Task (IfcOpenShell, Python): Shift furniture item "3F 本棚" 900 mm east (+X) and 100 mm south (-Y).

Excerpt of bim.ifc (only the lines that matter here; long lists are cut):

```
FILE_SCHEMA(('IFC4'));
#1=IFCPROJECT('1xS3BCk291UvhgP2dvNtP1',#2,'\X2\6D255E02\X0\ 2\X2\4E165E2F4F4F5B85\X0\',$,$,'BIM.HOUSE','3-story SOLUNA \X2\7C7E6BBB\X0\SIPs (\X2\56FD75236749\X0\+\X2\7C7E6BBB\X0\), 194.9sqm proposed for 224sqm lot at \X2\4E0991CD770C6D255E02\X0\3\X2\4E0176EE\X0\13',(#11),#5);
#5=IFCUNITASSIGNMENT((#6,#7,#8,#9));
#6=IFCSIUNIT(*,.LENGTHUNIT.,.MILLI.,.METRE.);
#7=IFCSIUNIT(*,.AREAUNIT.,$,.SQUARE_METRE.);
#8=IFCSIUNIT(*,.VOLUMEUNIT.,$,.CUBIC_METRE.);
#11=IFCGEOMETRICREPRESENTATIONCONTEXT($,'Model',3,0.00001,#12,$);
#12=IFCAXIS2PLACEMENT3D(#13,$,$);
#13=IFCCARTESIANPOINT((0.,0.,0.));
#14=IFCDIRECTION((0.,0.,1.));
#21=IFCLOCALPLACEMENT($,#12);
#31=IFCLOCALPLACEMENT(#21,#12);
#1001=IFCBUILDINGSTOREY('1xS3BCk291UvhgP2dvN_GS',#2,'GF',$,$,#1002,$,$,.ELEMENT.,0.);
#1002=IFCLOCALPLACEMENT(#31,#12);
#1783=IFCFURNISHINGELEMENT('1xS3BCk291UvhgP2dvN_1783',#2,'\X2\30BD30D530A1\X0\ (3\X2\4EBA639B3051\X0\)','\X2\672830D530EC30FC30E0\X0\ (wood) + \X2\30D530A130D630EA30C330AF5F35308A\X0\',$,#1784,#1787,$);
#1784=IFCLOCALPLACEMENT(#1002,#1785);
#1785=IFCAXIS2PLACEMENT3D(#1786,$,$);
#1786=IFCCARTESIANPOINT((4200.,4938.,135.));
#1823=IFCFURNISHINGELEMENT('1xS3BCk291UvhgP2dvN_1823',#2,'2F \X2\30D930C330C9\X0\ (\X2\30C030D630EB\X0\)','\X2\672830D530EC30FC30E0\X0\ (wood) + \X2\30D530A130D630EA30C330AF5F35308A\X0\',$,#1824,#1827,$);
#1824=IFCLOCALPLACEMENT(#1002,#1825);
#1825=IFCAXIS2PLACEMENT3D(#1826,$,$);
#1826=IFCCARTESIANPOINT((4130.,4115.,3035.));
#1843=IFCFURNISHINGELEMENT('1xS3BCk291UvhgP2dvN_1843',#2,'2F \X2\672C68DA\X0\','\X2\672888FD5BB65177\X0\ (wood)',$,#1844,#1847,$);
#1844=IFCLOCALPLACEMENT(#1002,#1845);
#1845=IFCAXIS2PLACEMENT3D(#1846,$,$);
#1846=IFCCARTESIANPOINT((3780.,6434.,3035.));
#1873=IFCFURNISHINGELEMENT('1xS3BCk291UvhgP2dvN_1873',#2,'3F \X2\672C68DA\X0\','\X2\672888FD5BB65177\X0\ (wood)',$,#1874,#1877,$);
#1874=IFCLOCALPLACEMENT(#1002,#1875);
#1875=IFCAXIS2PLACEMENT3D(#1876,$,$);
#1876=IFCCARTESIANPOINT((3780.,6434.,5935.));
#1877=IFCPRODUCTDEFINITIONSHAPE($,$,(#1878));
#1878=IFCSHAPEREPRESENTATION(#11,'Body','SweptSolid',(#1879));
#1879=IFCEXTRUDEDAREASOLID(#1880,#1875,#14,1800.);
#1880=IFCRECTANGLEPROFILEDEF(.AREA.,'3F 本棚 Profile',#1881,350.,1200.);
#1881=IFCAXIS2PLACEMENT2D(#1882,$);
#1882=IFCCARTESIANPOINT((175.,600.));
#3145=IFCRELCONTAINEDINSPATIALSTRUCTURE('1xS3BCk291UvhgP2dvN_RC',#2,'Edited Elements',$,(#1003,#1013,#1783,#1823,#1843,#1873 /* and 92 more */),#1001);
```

```python
import ifcopenshell
import ifcopenshell.api.geometry
import ifcopenshell.util.placement

model = ifcopenshell.open("bim.ifc")

item = model.by_id(1873)
matrix = ifcopenshell.util.placement.get_local_placement(item.ObjectPlacement)
matrix[0, 3] += 900.0
matrix[1, 3] -= 100.0
ifcopenshell.api.geometry.edit_object_placement(model, product=item, matrix=matrix, is_si=False)

print(ifcopenshell.util.placement.get_local_placement(item.ObjectPlacement).round(3) + 0.0)

model.write("bim_rev.ifc")
```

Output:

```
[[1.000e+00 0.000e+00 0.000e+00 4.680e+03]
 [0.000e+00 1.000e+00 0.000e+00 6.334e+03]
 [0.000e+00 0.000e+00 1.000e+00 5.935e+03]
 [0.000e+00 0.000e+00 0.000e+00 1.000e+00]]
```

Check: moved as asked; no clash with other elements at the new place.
